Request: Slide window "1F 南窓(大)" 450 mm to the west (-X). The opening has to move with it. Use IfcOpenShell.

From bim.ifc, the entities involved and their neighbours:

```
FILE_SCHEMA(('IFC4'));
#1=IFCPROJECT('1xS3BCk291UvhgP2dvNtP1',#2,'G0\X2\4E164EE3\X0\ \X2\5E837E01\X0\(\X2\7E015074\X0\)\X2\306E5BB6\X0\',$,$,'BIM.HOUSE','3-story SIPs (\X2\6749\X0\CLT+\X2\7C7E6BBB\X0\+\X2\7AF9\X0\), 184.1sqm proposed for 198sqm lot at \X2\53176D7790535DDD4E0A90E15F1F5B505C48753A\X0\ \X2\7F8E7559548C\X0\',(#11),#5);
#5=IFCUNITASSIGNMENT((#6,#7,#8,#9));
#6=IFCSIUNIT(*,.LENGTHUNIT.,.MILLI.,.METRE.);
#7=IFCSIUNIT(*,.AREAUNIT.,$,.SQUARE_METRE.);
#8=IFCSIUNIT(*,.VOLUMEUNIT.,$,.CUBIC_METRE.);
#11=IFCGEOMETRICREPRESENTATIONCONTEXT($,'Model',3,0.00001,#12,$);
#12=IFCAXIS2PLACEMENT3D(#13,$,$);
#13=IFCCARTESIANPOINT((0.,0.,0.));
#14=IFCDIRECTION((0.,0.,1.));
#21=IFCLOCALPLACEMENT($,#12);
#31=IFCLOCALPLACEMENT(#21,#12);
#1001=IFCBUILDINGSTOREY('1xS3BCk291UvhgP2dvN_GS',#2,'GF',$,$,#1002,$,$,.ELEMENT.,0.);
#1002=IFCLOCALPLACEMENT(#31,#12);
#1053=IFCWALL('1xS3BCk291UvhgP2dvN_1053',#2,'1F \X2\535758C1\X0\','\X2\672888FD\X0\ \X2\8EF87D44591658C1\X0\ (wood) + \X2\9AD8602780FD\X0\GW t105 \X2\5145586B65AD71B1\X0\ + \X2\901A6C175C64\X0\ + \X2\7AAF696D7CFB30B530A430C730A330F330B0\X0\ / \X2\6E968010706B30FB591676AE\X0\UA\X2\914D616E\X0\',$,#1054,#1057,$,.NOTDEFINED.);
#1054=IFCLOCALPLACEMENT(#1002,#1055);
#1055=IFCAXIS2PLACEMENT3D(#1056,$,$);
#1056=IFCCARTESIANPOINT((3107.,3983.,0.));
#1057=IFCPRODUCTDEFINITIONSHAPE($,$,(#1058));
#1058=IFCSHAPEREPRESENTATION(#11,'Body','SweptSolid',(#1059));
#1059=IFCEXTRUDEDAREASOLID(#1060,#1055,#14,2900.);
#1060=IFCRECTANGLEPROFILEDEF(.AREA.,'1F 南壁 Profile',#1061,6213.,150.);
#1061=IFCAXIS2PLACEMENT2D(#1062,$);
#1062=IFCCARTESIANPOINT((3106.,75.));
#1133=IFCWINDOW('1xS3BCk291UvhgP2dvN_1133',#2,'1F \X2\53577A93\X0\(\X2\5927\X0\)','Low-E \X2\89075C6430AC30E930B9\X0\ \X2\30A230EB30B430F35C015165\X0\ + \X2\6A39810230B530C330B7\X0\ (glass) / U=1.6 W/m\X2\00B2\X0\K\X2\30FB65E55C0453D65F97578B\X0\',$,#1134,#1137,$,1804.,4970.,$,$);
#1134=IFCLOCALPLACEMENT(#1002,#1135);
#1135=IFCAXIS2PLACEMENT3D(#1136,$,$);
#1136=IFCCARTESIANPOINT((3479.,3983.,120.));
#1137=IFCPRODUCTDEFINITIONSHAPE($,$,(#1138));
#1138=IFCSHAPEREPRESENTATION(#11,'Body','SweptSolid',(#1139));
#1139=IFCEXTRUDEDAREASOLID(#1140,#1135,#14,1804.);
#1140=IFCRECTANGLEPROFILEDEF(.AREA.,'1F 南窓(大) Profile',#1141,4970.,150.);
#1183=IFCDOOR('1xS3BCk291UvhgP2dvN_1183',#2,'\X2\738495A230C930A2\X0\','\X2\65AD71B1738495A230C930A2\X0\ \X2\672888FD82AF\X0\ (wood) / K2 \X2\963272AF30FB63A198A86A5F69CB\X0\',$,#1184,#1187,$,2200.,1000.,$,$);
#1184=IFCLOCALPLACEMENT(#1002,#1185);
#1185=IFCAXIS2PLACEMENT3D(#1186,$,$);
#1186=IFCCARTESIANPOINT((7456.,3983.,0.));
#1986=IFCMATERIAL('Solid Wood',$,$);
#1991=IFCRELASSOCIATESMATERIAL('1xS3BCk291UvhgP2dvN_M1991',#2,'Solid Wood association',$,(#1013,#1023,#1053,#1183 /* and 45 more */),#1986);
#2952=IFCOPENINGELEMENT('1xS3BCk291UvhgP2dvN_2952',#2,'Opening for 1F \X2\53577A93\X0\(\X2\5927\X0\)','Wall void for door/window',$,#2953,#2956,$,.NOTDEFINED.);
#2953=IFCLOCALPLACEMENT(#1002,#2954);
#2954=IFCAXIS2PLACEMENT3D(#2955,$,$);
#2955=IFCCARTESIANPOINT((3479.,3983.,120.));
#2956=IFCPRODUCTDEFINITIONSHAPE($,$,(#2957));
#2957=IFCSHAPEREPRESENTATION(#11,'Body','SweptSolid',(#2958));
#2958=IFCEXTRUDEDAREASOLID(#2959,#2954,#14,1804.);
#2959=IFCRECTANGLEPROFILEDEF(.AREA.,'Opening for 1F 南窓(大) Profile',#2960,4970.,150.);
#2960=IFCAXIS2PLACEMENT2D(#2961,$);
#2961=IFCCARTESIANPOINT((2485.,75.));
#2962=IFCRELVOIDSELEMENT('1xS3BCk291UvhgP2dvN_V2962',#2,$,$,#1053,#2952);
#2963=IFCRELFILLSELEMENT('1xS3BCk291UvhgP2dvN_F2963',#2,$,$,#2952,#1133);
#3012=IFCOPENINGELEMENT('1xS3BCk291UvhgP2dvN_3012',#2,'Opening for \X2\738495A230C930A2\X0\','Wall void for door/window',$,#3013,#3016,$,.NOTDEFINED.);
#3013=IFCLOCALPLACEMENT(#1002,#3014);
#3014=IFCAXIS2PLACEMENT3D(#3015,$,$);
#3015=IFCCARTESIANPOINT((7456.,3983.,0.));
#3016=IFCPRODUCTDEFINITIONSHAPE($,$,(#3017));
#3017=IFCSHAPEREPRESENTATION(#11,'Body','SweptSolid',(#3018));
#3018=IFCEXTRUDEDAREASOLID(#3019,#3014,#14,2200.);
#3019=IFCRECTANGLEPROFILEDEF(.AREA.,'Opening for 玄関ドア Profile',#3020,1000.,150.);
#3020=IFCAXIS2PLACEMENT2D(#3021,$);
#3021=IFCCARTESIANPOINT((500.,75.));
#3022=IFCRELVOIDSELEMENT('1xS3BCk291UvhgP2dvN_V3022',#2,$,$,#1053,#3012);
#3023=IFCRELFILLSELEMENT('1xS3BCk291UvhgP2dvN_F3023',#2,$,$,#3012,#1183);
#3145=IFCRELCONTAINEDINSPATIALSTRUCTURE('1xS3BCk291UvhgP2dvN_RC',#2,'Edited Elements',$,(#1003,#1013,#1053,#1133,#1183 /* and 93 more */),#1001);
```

```python
import ifcopenshell
import ifcopenshell.api.geometry
import ifcopenshell.util.placement
import ifcopenshell.util.unit

model = ifcopenshell.open("bim.ifc")
unit_scale = ifcopenshell.util.unit.calculate_unit_scale(model)

window = model.by_guid("1xS3BCk291UvhgP2dvN_1133")
opening = window.FillsVoids[0].RelatingOpeningElement
wall = opening.VoidsElements[0].RelatingBuildingElement

wall_matrix = ifcopenshell.util.placement.get_local_placement(wall.ObjectPlacement)
shift = wall_matrix[:3, 0] * -0.45 / unit_scale
before = ifcopenshell.util.placement.get_local_placement(window.ObjectPlacement)[:3, 3].copy()

# The window is not placed relative to its opening, so move both.
for product in (opening, window):
    matrix = ifcopenshell.util.placement.get_local_placement(product.ObjectPlacement)
    matrix[:3, 3] += shift
    ifcopenshell.api.geometry.edit_object_placement(model, product=product, matrix=matrix, is_si=False)

after = ifcopenshell.util.placement.get_local_placement(window.ObjectPlacement)[:3, 3]
print("window moved by", (after - before).round(3) + 0.0)

model.write("bim-out.ifc")
```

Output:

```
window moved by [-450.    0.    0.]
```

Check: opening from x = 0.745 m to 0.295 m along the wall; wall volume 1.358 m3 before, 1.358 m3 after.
